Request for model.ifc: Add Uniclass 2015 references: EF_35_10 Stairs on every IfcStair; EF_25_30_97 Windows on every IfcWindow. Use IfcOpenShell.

First a look at what the model holds.

```python
import ifcopenshell

model = ifcopenshell.open("model.ifc")
print(model.schema)
print("classifications:", [c.Name for c in model.by_type("IfcClassification")])
for ifc_class in ("IfcDoor", "IfcRoof", "IfcStair", "IfcWall", "IfcWindow"):
    print(ifc_class, len(model.by_type(ifc_class)))
```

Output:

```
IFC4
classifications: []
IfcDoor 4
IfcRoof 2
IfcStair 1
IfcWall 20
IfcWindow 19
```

```python
import ifcopenshell
import ifcopenshell.api.classification

model = ifcopenshell.open("model.ifc")

system = ifcopenshell.api.classification.add_classification(model, classification="Uniclass 2015")

codes = {
    "IfcStair": ("EF_35_10", "Stairs"),
    "IfcWindow": ("EF_25_30_97", "Windows"),
}
for ifc_class, (code, name) in codes.items():
    products = model.by_type(ifc_class)
    ifcopenshell.api.classification.add_reference(
        model, products=products, classification=system, identification=code, name=name
    )
    print(code, len(products))

model.write("model_rev.ifc")
```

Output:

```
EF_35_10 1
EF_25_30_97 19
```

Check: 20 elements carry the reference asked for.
